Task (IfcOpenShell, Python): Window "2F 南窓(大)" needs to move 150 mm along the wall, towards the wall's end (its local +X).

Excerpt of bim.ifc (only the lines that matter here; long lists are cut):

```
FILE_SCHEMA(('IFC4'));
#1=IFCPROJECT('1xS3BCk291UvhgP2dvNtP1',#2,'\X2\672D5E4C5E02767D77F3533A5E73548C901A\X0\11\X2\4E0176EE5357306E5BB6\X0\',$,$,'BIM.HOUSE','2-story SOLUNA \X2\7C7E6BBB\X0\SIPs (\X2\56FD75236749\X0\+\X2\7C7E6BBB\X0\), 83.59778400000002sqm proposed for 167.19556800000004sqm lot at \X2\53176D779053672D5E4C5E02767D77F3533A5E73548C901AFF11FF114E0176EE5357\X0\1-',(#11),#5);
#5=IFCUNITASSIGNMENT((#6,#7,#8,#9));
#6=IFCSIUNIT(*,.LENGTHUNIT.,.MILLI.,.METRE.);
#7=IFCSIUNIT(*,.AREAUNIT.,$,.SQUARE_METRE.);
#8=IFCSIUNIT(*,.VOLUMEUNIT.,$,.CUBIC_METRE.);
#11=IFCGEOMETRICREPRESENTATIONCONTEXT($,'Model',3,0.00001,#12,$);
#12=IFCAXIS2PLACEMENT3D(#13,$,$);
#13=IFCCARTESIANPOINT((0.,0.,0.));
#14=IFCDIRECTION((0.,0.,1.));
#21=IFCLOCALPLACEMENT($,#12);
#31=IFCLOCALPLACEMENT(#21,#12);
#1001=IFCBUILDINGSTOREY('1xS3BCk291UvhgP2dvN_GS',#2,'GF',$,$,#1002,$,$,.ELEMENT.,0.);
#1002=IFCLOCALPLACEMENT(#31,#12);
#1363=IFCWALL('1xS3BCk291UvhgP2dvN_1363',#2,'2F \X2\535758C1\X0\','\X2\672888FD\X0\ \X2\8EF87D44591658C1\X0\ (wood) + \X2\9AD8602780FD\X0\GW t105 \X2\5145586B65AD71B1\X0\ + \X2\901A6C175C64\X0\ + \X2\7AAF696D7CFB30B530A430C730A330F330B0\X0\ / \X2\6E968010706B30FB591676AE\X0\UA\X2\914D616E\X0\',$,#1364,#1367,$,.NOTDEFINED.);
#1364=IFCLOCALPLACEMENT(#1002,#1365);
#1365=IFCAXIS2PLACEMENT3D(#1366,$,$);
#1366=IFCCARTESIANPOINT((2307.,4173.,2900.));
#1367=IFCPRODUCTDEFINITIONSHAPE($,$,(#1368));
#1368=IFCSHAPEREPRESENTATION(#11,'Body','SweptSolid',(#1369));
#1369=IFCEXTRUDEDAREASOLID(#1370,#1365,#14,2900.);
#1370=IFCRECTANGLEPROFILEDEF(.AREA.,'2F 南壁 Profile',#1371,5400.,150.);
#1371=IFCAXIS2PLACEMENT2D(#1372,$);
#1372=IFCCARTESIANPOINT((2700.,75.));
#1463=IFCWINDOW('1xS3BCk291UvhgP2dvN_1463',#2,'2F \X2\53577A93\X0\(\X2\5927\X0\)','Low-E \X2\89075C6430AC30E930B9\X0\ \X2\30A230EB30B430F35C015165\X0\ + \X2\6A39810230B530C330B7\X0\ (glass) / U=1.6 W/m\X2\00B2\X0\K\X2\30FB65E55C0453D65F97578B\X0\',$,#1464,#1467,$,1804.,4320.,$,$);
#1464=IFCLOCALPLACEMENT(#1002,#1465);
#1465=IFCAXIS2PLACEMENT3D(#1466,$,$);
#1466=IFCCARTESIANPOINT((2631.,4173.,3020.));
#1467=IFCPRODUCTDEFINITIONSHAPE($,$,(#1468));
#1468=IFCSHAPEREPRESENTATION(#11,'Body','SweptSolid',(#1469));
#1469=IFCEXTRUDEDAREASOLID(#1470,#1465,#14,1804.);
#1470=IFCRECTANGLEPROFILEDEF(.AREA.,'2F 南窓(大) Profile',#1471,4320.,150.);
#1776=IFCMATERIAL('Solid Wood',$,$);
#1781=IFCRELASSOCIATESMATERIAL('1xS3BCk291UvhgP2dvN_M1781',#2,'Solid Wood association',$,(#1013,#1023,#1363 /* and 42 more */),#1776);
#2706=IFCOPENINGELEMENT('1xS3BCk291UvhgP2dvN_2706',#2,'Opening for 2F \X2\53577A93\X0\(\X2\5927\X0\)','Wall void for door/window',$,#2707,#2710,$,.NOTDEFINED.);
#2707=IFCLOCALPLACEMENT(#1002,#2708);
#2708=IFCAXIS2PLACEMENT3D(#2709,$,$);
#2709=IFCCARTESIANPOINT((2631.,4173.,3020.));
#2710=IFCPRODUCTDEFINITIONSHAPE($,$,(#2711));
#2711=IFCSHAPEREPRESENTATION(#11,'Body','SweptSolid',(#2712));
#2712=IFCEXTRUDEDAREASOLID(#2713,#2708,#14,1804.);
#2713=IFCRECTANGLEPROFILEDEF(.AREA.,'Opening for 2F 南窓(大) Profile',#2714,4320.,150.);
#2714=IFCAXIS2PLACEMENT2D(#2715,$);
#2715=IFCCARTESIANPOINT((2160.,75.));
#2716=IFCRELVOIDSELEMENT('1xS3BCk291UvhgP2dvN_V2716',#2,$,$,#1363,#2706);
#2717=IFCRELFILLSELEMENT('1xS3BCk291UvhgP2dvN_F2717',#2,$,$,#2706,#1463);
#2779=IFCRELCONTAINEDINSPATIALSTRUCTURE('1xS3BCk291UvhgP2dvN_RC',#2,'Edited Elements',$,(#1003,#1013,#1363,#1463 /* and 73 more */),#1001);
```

```python
import ifcopenshell
import ifcopenshell.api.geometry
import ifcopenshell.util.placement

model = ifcopenshell.open("bim.ifc")

window = model.by_guid("1xS3BCk291UvhgP2dvN_1463")
opening = window.FillsVoids[0].RelatingOpeningElement
wall = opening.VoidsElements[0].RelatingBuildingElement

wall_matrix = ifcopenshell.util.placement.get_local_placement(wall.ObjectPlacement)
shift = wall_matrix[:3, 0] * 150.0
before = ifcopenshell.util.placement.get_local_placement(window.ObjectPlacement)[:3, 3].copy()

# The window is not placed relative to its opening, so move both.
for product in (opening, window):
    matrix = ifcopenshell.util.placement.get_local_placement(product.ObjectPlacement)
    matrix[:3, 3] += shift
    ifcopenshell.api.geometry.edit_object_placement(model, product=product, matrix=matrix, is_si=False)

after = ifcopenshell.util.placement.get_local_placement(window.ObjectPlacement)[:3, 3]
print("window moved by", (after - before).round(3) + 0.0)

model.write("bim_rev.ifc")
```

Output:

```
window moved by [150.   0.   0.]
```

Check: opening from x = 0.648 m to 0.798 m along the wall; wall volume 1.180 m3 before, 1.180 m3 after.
